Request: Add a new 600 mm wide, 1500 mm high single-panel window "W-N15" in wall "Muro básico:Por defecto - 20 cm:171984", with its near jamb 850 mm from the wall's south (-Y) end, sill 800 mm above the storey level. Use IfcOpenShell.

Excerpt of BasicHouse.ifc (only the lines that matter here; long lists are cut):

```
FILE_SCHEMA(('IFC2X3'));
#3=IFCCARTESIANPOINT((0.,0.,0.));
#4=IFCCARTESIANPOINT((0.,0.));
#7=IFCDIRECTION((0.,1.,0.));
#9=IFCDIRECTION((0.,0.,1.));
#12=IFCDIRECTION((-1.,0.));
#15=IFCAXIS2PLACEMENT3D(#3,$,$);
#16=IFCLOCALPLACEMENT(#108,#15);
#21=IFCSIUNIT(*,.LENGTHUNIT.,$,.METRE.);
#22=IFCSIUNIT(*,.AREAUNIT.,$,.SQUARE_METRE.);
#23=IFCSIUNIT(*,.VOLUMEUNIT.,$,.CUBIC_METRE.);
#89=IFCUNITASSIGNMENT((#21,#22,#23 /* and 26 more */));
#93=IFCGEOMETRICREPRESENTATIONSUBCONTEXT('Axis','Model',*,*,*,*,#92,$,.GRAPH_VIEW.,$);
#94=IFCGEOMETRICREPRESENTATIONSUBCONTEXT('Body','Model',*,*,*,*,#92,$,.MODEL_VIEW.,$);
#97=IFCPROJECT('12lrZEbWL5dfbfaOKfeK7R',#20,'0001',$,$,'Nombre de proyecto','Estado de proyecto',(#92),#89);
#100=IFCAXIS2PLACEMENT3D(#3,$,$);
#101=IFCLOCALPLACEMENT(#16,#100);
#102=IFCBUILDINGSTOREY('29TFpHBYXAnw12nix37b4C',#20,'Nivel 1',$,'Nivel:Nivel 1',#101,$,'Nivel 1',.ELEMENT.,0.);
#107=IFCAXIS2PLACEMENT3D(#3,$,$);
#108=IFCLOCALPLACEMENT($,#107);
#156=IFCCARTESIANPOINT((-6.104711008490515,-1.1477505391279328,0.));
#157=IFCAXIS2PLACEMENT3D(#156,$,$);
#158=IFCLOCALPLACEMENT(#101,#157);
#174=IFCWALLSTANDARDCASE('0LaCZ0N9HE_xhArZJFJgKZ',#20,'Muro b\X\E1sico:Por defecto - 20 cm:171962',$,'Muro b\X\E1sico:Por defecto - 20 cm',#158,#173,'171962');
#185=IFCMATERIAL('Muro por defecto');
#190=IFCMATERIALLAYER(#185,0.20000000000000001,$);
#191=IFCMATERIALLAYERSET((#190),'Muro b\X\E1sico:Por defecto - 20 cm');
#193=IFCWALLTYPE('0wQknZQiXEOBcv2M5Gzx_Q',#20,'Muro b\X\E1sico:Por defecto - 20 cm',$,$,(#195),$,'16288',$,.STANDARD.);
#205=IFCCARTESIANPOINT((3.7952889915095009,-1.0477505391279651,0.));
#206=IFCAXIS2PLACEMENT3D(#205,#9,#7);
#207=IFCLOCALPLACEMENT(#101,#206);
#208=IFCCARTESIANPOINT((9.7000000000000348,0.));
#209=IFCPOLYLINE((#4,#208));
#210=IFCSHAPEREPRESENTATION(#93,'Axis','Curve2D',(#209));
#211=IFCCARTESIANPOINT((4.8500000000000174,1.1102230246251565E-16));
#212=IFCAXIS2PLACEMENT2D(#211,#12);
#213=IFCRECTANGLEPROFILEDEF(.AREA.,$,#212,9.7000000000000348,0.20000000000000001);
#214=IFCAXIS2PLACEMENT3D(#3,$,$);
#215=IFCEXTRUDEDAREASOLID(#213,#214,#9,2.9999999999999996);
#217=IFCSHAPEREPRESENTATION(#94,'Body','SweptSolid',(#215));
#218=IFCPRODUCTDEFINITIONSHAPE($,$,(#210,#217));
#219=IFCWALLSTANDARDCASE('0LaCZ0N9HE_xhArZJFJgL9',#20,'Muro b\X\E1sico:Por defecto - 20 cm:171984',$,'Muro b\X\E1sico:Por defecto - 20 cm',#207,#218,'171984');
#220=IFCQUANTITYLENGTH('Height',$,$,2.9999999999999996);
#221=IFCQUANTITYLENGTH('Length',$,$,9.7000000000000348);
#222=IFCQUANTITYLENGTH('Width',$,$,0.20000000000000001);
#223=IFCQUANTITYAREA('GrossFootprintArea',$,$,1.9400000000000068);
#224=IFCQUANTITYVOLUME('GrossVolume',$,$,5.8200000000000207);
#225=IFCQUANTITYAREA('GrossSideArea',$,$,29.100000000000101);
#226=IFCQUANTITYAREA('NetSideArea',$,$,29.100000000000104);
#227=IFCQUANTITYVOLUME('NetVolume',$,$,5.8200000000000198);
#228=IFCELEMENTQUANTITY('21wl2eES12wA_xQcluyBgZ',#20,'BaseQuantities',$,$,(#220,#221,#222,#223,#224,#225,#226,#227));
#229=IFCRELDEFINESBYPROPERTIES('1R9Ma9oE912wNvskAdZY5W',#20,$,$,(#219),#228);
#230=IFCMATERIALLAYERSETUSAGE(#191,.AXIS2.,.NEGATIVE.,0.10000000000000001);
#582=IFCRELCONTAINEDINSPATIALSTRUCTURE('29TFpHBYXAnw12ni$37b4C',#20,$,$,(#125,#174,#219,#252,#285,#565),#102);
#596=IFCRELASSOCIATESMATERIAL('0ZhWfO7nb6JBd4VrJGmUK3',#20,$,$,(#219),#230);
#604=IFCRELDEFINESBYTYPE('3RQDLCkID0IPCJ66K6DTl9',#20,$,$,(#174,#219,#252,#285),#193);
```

```python
import numpy as np
import ifcopenshell
import ifcopenshell.api.feature
import ifcopenshell.api.geometry
import ifcopenshell.api.pset
import ifcopenshell.api.root
import ifcopenshell.api.spatial
import ifcopenshell.api.type
import ifcopenshell.geom
import ifcopenshell.util.element
import ifcopenshell.util.placement
import ifcopenshell.util.representation
import ifcopenshell.util.shape
import ifcopenshell.util.unit

model = ifcopenshell.open("BasicHouse.ifc")
unit_scale = ifcopenshell.util.unit.calculate_unit_scale(model)
area_scale = ifcopenshell.util.unit.calculate_unit_scale(model, "AREAUNIT")
volume_scale = ifcopenshell.util.unit.calculate_unit_scale(model, "VOLUMEUNIT")
settings = ifcopenshell.geom.settings()


def volume(element):
    """Net volume in cubic metres, openings subtracted."""
    shape = ifcopenshell.geom.create_shape(settings, element)
    return ifcopenshell.util.shape.get_volume(shape.geometry)


wall = model.by_id(219)
storey = ifcopenshell.util.element.get_container(wall, ifc_class="IfcBuildingStorey")
context = ifcopenshell.util.representation.get_context(model, "Model", "Body", "MODEL_VIEW")
before = volume(wall)

width, height, from_end, sill = 0.6, 1.5, 0.85, 0.8  # metres

# The wall runs along its own X axis, and the end named is its -X end.
wall_shape = ifcopenshell.geom.create_shape(settings, wall)
x, y, z = ifcopenshell.util.shape.get_vertices(wall_shape.geometry).T
start = x.min() + from_end
face, thickness = float(y.min()), float(y.max() - y.min())
wall_matrix = ifcopenshell.util.placement.get_local_placement(wall.ObjectPlacement)
level = ifcopenshell.util.placement.get_local_placement(storey.ObjectPlacement)[2, 3]


def in_wall(x, y):
    """Placement at x, y metres in the wall's axes, at sill height."""
    matrix = wall_matrix.copy()
    matrix[:, 3] = wall_matrix @ np.array([x / unit_scale, y / unit_scale, 0.0, 1.0])
    matrix[2, 3] = level + sill / unit_scale
    return matrix


# Opening: a box that overshoots both wall faces by 50 mm.
opening = ifcopenshell.api.root.create_entity(model, ifc_class="IfcOpeningElement")
box = ifcopenshell.api.geometry.add_wall_representation(
    model, context=context, length=width, height=height, thickness=thickness + 0.1
)
ifcopenshell.api.geometry.assign_representation(model, product=opening, representation=box)
ifcopenshell.api.geometry.edit_object_placement(model, product=opening, matrix=in_wall(start, face - 0.05), is_si=False)
ifcopenshell.api.feature.add_feature(model, feature=opening, element=wall)

window = ifcopenshell.api.root.create_entity(model, ifc_class="IfcWindow", name="W-N15")
window.OverallWidth, window.OverallHeight = width / unit_scale, height / unit_scale
body = ifcopenshell.api.geometry.add_window_representation(
    model,
    context=context,
    overall_width=window.OverallWidth,
    overall_height=window.OverallHeight,
    partition_type="SINGLE_PANEL",
)
ifcopenshell.api.geometry.assign_representation(model, product=window, representation=body)
ifcopenshell.api.spatial.assign_container(model, products=[window], relating_structure=storey)
fills = ifcopenshell.api.feature.add_filling(model, opening=opening, element=window)
fills.OwnerHistory = window.OwnerHistory  # required in IFC2X3

# IFC2X3 keeps the operation on the window style.
style = ifcopenshell.api.root.create_entity(model, ifc_class="IfcWindowStyle", name="W-N15")
style.OperationType, style.ConstructionType = "SINGLE_PANEL", "NOTDEFINED"
style.ParameterTakesPrecedence = style.Sizeable = False
ifcopenshell.api.type.assign_type(model, related_objects=[window], relating_type=style)

# Centre the window in the wall's thickness.
ifcopenshell.api.geometry.edit_object_placement(model, product=window, matrix=in_wall(start, face), is_si=False)
window_shape = ifcopenshell.geom.create_shape(settings, window)
depth = ifcopenshell.util.shape.get_vertices(window_shape.geometry)[:, 1]
offset = face + thickness / 2 - (depth.min() + depth.max()) / 2
ifcopenshell.api.geometry.edit_object_placement(model, product=window, matrix=in_wall(start, offset), is_si=False)

after = volume(wall)

# Update the wall's stored quantities.
qto = model.by_id(ifcopenshell.util.element.get_pset(wall, "BaseQuantities", should_inherit=False)["id"])
ifcopenshell.api.pset.edit_qto(model, qto=qto, properties={
    "NetSideArea": after / thickness / area_scale,
    "NetVolume": after / volume_scale,
})

print(f"wall volume {before:.3f} -> {after:.3f} m3")

model.write("BasicHouse_rev.ifc")
```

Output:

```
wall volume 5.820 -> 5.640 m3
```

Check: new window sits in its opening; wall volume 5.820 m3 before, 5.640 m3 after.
